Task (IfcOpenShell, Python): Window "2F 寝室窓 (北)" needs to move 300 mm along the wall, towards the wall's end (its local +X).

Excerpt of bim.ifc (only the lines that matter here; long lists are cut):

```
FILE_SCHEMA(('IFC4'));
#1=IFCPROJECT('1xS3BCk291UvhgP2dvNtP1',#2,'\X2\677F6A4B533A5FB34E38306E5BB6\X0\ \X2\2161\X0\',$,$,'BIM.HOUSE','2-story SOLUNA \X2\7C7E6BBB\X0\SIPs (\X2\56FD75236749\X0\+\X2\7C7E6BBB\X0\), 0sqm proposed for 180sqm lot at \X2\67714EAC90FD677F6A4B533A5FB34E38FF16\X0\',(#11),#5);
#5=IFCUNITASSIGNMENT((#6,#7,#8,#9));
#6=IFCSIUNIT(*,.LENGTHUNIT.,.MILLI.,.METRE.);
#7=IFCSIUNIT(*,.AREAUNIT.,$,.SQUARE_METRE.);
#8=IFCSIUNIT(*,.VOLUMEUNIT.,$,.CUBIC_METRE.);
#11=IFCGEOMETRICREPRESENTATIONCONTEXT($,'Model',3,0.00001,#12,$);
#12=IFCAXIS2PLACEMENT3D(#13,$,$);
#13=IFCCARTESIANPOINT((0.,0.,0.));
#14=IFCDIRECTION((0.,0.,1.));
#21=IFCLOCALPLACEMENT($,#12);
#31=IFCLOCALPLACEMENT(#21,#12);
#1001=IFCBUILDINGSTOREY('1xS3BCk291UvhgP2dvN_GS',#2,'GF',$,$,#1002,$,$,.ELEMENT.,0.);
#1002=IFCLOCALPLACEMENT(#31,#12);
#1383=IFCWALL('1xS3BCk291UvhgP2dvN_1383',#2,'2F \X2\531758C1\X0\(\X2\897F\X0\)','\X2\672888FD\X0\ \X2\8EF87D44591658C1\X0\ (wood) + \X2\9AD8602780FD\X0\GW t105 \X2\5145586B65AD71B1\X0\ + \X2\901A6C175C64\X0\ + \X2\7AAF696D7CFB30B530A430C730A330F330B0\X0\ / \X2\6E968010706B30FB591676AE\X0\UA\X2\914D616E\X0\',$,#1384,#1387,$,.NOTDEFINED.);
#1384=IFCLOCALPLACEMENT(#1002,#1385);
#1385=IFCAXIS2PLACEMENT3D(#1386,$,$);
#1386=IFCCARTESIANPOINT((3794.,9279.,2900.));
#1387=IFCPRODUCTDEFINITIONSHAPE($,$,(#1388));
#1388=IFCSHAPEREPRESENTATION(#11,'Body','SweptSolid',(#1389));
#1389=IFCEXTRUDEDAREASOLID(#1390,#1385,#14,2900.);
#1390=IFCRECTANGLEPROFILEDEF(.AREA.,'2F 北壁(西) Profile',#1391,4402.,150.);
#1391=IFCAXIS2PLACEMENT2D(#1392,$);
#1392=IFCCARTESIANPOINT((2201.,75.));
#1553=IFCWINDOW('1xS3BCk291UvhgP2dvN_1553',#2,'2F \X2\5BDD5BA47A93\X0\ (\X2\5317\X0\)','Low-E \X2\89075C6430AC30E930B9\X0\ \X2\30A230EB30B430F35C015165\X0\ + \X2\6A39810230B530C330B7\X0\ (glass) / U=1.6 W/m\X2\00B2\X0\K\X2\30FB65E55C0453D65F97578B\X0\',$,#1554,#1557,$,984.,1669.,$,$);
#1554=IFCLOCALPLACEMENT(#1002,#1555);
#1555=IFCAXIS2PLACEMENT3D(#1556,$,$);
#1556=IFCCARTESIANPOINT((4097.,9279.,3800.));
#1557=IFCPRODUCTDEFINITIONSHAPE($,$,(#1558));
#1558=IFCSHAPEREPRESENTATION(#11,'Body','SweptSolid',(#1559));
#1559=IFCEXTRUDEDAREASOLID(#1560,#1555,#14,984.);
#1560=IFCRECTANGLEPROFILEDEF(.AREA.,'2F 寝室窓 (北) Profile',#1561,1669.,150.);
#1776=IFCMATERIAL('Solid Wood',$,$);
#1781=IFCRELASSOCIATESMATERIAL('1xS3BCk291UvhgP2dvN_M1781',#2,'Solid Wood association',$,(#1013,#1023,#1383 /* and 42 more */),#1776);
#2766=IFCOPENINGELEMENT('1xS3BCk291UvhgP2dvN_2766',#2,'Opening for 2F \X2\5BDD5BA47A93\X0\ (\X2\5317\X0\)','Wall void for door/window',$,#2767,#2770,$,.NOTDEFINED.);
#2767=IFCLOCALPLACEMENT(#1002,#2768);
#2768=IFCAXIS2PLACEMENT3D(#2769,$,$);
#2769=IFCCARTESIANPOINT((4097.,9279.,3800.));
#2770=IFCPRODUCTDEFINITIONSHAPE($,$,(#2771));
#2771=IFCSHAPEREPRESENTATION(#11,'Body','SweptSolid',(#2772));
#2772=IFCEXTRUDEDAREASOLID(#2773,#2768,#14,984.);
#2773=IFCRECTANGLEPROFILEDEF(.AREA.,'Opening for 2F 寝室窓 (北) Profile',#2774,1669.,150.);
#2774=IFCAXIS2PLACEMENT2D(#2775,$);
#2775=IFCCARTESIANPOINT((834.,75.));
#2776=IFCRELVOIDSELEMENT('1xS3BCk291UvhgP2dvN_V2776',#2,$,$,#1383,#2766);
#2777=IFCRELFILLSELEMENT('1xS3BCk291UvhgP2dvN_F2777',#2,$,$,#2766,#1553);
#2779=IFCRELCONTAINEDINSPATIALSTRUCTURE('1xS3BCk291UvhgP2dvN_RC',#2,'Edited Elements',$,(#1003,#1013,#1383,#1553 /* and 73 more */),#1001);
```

```python
import ifcopenshell
import ifcopenshell.api.geometry
import ifcopenshell.util.placement

model = ifcopenshell.open("bim.ifc")

window = model.by_guid("1xS3BCk291UvhgP2dvN_1553")
opening = window.FillsVoids[0].RelatingOpeningElement
wall = opening.VoidsElements[0].RelatingBuildingElement

wall_matrix = ifcopenshell.util.placement.get_local_placement(wall.ObjectPlacement)
shift = wall_matrix[:3, 0] * 300.0
before = ifcopenshell.util.placement.get_local_placement(window.ObjectPlacement)[:3, 3].copy()

# The window is not placed relative to its opening, so move both.
for product in (opening, window):
    matrix = ifcopenshell.util.placement.get_local_placement(product.ObjectPlacement)
    matrix[:3, 3] += shift
    ifcopenshell.api.geometry.edit_object_placement(model, product=product, matrix=matrix, is_si=False)

after = ifcopenshell.util.placement.get_local_placement(window.ObjectPlacement)[:3, 3]
print("window moved by", (after - before).round(3) + 0.0)

model.write("bim_v2.ifc")
```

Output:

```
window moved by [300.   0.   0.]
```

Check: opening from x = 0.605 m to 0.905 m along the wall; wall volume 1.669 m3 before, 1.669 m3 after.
